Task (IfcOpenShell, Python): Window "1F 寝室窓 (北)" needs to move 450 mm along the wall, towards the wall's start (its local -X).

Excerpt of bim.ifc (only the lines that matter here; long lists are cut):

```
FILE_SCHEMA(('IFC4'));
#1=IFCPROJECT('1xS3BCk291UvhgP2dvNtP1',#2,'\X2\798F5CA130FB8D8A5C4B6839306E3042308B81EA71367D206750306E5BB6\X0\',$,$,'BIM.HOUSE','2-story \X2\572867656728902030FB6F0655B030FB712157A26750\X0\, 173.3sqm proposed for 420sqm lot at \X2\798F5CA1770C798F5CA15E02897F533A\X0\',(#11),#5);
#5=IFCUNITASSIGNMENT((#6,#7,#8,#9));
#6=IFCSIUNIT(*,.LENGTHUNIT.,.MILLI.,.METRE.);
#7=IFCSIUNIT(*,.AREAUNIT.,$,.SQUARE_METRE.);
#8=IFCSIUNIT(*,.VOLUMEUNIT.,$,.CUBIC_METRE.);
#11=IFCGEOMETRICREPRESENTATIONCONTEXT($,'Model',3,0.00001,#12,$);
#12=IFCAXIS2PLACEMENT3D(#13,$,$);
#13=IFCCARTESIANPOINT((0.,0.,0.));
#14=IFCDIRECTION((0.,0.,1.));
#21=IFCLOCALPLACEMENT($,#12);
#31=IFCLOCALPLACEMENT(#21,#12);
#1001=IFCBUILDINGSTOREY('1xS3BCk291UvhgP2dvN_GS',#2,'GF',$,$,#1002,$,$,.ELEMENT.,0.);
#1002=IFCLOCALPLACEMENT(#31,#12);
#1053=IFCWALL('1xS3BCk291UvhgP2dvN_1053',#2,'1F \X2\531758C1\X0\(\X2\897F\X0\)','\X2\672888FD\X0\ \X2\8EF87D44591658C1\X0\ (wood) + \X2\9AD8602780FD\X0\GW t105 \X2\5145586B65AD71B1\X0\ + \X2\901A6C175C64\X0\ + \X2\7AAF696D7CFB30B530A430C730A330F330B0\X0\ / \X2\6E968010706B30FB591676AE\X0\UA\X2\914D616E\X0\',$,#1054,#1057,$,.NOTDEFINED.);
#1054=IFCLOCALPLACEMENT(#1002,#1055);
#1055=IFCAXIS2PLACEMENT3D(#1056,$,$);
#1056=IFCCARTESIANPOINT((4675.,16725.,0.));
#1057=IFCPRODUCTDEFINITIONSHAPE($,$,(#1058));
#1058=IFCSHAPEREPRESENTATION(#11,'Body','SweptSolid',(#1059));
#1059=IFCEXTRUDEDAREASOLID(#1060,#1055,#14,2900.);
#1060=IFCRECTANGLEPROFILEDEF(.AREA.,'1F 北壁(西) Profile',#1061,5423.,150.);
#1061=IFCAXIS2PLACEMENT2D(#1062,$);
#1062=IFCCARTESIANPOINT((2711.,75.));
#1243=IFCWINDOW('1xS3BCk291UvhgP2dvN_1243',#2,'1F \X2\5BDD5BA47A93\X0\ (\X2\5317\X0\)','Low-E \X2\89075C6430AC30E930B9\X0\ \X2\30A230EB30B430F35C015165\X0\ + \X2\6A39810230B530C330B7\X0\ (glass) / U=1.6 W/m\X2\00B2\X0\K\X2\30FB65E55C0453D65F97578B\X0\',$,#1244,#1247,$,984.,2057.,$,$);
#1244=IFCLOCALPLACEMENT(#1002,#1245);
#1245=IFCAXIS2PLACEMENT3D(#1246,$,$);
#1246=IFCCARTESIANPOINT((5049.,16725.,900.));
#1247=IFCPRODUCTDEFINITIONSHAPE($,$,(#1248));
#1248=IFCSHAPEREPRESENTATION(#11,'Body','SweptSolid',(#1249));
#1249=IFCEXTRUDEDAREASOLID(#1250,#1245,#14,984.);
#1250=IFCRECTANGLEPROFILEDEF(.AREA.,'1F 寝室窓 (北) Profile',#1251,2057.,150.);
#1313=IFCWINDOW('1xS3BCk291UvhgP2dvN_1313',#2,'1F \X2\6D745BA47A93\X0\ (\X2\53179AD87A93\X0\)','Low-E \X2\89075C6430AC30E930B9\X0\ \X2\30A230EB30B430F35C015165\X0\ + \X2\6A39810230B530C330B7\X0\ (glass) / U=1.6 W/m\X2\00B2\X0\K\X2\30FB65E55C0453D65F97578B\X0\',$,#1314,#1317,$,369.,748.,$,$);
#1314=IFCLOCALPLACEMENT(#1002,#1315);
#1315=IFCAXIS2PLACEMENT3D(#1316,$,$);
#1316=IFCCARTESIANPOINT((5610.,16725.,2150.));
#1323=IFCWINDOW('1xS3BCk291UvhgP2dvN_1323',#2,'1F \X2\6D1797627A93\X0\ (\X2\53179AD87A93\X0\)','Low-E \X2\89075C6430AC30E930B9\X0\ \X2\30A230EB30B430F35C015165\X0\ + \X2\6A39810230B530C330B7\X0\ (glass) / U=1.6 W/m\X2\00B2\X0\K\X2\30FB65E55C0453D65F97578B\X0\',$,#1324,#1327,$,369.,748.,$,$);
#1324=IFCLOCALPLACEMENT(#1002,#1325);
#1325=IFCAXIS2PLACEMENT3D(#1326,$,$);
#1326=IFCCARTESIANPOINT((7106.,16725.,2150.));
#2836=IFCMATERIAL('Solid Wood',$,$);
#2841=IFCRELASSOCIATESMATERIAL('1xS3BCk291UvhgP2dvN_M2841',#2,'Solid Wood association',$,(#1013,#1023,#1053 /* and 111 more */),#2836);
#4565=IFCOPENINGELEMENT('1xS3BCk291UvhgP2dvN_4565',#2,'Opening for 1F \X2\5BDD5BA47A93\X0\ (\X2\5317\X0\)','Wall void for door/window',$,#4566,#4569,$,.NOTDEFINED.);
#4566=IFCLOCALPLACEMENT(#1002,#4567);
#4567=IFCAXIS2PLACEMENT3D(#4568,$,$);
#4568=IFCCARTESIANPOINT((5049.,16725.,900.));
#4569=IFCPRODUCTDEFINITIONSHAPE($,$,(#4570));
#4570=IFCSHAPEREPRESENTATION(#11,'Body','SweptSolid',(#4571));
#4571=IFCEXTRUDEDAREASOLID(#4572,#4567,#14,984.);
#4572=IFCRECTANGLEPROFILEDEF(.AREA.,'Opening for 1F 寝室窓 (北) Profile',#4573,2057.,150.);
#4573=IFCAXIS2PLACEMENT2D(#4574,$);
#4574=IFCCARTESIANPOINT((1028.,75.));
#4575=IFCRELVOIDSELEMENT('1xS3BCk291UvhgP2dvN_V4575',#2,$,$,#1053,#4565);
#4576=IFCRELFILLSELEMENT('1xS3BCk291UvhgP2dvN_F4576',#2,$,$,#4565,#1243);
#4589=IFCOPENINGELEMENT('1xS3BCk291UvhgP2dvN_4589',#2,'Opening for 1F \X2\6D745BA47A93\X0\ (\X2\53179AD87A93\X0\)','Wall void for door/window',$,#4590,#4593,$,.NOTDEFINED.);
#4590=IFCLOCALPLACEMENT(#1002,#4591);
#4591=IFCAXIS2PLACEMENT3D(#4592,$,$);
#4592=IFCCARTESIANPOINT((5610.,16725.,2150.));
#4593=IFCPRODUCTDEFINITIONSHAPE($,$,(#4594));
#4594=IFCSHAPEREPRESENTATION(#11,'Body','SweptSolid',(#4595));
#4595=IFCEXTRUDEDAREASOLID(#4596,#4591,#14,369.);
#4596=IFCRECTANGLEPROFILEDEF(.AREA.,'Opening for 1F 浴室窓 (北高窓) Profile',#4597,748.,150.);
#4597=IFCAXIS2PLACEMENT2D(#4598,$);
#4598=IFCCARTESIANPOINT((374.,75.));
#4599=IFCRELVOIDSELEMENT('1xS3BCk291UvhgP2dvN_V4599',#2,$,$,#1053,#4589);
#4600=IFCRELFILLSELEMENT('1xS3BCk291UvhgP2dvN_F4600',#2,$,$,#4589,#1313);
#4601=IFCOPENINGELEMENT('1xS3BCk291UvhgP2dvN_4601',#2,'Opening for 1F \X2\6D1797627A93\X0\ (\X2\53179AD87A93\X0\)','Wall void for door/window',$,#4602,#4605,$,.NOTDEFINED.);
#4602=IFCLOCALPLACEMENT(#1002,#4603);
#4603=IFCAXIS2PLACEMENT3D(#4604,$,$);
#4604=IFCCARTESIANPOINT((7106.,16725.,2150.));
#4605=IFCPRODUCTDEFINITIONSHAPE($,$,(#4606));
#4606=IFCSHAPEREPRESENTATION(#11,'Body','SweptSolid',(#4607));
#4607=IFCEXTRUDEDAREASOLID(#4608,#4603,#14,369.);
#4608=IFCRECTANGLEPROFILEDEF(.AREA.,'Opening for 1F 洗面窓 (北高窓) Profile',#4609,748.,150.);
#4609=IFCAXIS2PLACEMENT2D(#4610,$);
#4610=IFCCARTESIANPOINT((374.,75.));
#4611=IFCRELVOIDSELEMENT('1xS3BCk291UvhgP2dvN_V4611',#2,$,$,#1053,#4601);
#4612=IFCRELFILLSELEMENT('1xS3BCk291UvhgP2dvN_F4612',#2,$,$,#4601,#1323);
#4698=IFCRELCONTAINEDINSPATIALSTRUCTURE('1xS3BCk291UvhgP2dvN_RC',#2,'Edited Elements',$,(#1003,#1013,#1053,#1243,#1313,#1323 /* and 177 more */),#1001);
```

```python
import ifcopenshell
import ifcopenshell.api.geometry
import ifcopenshell.util.placement
import ifcopenshell.util.unit

model = ifcopenshell.open("bim.ifc")
unit_scale = ifcopenshell.util.unit.calculate_unit_scale(model)

window = model.by_guid("1xS3BCk291UvhgP2dvN_1243")
opening = window.FillsVoids[0].RelatingOpeningElement
wall = opening.VoidsElements[0].RelatingBuildingElement

wall_matrix = ifcopenshell.util.placement.get_local_placement(wall.ObjectPlacement)
shift = wall_matrix[:3, 0] * -0.45 / unit_scale
before = ifcopenshell.util.placement.get_local_placement(window.ObjectPlacement)[:3, 3].copy()

# The window is not placed relative to its opening, so move both.
for product in (opening, window):
    matrix = ifcopenshell.util.placement.get_local_placement(product.ObjectPlacement)
    matrix[:3, 3] += shift
    ifcopenshell.api.geometry.edit_object_placement(model, product=product, matrix=matrix, is_si=False)

after = ifcopenshell.util.placement.get_local_placement(window.ObjectPlacement)[:3, 3]
print("window moved by", (after - before).round(3) + 0.0)

model.write("bim_rev.ifc")
```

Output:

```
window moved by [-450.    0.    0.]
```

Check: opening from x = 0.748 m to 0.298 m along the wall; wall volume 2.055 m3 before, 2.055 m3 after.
